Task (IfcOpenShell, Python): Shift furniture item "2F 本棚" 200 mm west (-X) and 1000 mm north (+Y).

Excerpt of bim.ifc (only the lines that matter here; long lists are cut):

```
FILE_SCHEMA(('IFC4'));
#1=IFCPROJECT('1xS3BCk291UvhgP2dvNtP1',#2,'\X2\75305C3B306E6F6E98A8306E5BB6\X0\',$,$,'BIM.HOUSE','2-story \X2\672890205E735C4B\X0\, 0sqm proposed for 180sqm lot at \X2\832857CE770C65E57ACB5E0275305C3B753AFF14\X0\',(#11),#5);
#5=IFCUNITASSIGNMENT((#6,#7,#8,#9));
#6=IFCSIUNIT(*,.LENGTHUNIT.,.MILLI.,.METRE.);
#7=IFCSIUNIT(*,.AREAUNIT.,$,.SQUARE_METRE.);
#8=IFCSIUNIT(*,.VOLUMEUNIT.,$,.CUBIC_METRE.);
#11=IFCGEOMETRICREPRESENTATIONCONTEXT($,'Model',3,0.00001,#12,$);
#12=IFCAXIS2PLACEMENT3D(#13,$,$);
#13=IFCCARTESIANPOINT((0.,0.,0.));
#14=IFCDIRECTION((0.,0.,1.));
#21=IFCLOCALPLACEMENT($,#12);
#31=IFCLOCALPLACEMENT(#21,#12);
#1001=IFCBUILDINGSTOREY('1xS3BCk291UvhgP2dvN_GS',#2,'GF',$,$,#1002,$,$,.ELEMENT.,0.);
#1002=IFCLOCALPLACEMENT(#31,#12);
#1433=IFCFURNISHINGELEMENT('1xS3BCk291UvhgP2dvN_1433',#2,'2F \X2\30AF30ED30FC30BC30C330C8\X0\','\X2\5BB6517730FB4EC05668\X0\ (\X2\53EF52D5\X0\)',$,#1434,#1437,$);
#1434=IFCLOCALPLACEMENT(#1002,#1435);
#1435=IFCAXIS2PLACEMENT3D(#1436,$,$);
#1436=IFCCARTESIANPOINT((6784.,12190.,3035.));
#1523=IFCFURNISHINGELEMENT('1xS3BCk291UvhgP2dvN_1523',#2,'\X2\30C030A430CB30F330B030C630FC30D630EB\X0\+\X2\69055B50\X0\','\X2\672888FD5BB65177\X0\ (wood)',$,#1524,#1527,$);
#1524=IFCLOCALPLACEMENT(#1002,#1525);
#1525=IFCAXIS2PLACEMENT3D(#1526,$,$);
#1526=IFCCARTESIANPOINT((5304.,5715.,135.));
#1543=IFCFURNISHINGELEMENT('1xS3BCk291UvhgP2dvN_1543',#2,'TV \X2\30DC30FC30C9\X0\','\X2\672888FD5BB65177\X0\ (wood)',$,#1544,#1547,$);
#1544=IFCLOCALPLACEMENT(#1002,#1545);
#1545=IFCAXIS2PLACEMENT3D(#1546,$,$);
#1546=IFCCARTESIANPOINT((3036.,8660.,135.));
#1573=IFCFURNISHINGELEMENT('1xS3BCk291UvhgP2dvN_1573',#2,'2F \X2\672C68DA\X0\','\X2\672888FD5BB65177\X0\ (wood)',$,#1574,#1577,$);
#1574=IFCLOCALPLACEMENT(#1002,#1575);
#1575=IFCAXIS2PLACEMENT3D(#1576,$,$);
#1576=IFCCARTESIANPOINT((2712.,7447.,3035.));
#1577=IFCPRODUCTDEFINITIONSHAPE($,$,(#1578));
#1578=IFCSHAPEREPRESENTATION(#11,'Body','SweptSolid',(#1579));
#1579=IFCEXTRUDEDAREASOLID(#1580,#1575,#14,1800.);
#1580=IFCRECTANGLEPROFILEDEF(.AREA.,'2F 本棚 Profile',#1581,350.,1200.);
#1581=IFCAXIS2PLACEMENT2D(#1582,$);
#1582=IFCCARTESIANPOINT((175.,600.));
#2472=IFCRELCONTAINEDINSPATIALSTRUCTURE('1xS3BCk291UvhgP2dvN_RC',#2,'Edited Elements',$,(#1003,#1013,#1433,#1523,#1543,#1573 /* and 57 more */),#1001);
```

```python
import ifcopenshell
import ifcopenshell.api.geometry
import ifcopenshell.util.placement

model = ifcopenshell.open("bim.ifc")

item = model.by_id(1573)
matrix = ifcopenshell.util.placement.get_local_placement(item.ObjectPlacement)
matrix[0, 3] -= 200.0
matrix[1, 3] += 1000.0
ifcopenshell.api.geometry.edit_object_placement(model, product=item, matrix=matrix, is_si=False)

print(ifcopenshell.util.placement.get_local_placement(item.ObjectPlacement).round(3) + 0.0)

model.write("bim_updated.ifc")
```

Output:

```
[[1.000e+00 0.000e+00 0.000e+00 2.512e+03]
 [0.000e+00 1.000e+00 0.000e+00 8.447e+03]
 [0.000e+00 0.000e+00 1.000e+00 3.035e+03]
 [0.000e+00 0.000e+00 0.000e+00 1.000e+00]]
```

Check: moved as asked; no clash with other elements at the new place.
